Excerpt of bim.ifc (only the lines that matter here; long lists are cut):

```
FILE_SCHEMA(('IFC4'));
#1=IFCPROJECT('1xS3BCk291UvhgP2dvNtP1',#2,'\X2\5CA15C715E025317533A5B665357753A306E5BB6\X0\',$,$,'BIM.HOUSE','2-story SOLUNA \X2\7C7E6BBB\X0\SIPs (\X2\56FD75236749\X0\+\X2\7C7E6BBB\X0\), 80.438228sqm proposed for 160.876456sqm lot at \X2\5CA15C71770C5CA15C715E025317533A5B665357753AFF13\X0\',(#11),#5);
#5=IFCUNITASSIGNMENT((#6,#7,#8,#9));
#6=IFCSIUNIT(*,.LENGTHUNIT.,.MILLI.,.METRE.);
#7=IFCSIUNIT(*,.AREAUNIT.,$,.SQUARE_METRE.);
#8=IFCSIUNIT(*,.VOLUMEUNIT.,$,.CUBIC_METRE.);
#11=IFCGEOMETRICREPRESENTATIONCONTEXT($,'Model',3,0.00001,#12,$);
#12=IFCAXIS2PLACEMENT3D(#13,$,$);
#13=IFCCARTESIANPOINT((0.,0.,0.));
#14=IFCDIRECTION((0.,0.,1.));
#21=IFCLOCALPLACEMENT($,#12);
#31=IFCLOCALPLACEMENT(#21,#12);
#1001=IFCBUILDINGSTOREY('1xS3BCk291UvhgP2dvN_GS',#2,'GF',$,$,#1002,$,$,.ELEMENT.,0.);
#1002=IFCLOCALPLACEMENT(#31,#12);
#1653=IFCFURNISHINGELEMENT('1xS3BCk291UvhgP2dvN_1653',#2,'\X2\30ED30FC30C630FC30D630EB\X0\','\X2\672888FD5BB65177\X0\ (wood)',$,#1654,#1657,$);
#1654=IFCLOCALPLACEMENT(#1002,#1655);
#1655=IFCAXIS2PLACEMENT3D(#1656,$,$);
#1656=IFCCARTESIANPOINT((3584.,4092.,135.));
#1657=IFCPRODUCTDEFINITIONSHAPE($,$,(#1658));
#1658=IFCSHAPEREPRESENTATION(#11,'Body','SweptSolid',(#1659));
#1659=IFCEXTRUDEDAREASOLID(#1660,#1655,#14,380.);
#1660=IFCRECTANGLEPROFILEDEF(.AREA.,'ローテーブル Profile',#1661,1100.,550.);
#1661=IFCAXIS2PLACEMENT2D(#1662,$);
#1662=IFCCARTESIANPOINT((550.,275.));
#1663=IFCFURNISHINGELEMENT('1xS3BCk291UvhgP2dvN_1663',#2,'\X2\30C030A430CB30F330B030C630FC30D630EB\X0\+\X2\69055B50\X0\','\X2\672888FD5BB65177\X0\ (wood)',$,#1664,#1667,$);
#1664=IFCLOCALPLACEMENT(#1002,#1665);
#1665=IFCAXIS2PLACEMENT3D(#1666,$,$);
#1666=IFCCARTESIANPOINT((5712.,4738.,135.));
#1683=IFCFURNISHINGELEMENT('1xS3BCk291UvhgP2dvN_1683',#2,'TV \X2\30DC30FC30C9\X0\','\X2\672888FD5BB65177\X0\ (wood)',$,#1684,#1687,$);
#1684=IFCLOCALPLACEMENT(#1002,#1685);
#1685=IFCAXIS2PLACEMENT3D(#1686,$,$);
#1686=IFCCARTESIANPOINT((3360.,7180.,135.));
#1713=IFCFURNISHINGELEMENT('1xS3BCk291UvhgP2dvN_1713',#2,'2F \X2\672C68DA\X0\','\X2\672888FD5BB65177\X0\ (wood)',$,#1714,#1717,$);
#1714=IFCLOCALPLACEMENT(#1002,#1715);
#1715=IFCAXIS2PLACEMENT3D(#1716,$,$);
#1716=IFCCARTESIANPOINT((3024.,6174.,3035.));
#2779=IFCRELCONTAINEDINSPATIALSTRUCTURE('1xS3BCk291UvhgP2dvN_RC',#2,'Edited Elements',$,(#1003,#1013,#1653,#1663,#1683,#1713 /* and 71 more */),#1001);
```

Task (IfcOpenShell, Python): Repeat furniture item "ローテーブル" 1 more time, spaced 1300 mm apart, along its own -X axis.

```python
import ifcopenshell
import ifcopenshell.api.geometry
import ifcopenshell.api.root
import ifcopenshell.util.element
import ifcopenshell.util.placement

model = ifcopenshell.open("bim.ifc")


def reuse_history(source, copy):
    """copy_class also copies each property set's owner history, people and application; keep the originals."""
    for rel in copy.IsDefinedBy:
        if rel.is_a("IfcRelDefinesByProperties") and (history := rel.RelatingPropertyDefinition.OwnerHistory):
            rel.RelatingPropertyDefinition.OwnerHistory = source.OwnerHistory
            ifcopenshell.util.element.remove_deep2(model, history)


source = model.by_guid("1xS3BCk291UvhgP2dvN_1653")
base = ifcopenshell.util.placement.get_local_placement(source.ObjectPlacement)
step = -base[:3, 0] * 1300.0

for i in range(1, 2):
    copy = ifcopenshell.api.root.copy_class(model, product=source)
    copy.Representation = ifcopenshell.util.element.copy_deep(
        model, source.Representation, exclude=["IfcGeometricRepresentationContext", "IfcRepresentationMap"]
    )
    reuse_history(source, copy)
    matrix = base.copy()
    matrix[:3, 3] += i * step
    print("added at", matrix[:3, 3].round(3) + 0.0)
    ifcopenshell.api.geometry.edit_object_placement(model, product=copy, matrix=matrix, is_si=False)

model.write("bim-out.ifc")
```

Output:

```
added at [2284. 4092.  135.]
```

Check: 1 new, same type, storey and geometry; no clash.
